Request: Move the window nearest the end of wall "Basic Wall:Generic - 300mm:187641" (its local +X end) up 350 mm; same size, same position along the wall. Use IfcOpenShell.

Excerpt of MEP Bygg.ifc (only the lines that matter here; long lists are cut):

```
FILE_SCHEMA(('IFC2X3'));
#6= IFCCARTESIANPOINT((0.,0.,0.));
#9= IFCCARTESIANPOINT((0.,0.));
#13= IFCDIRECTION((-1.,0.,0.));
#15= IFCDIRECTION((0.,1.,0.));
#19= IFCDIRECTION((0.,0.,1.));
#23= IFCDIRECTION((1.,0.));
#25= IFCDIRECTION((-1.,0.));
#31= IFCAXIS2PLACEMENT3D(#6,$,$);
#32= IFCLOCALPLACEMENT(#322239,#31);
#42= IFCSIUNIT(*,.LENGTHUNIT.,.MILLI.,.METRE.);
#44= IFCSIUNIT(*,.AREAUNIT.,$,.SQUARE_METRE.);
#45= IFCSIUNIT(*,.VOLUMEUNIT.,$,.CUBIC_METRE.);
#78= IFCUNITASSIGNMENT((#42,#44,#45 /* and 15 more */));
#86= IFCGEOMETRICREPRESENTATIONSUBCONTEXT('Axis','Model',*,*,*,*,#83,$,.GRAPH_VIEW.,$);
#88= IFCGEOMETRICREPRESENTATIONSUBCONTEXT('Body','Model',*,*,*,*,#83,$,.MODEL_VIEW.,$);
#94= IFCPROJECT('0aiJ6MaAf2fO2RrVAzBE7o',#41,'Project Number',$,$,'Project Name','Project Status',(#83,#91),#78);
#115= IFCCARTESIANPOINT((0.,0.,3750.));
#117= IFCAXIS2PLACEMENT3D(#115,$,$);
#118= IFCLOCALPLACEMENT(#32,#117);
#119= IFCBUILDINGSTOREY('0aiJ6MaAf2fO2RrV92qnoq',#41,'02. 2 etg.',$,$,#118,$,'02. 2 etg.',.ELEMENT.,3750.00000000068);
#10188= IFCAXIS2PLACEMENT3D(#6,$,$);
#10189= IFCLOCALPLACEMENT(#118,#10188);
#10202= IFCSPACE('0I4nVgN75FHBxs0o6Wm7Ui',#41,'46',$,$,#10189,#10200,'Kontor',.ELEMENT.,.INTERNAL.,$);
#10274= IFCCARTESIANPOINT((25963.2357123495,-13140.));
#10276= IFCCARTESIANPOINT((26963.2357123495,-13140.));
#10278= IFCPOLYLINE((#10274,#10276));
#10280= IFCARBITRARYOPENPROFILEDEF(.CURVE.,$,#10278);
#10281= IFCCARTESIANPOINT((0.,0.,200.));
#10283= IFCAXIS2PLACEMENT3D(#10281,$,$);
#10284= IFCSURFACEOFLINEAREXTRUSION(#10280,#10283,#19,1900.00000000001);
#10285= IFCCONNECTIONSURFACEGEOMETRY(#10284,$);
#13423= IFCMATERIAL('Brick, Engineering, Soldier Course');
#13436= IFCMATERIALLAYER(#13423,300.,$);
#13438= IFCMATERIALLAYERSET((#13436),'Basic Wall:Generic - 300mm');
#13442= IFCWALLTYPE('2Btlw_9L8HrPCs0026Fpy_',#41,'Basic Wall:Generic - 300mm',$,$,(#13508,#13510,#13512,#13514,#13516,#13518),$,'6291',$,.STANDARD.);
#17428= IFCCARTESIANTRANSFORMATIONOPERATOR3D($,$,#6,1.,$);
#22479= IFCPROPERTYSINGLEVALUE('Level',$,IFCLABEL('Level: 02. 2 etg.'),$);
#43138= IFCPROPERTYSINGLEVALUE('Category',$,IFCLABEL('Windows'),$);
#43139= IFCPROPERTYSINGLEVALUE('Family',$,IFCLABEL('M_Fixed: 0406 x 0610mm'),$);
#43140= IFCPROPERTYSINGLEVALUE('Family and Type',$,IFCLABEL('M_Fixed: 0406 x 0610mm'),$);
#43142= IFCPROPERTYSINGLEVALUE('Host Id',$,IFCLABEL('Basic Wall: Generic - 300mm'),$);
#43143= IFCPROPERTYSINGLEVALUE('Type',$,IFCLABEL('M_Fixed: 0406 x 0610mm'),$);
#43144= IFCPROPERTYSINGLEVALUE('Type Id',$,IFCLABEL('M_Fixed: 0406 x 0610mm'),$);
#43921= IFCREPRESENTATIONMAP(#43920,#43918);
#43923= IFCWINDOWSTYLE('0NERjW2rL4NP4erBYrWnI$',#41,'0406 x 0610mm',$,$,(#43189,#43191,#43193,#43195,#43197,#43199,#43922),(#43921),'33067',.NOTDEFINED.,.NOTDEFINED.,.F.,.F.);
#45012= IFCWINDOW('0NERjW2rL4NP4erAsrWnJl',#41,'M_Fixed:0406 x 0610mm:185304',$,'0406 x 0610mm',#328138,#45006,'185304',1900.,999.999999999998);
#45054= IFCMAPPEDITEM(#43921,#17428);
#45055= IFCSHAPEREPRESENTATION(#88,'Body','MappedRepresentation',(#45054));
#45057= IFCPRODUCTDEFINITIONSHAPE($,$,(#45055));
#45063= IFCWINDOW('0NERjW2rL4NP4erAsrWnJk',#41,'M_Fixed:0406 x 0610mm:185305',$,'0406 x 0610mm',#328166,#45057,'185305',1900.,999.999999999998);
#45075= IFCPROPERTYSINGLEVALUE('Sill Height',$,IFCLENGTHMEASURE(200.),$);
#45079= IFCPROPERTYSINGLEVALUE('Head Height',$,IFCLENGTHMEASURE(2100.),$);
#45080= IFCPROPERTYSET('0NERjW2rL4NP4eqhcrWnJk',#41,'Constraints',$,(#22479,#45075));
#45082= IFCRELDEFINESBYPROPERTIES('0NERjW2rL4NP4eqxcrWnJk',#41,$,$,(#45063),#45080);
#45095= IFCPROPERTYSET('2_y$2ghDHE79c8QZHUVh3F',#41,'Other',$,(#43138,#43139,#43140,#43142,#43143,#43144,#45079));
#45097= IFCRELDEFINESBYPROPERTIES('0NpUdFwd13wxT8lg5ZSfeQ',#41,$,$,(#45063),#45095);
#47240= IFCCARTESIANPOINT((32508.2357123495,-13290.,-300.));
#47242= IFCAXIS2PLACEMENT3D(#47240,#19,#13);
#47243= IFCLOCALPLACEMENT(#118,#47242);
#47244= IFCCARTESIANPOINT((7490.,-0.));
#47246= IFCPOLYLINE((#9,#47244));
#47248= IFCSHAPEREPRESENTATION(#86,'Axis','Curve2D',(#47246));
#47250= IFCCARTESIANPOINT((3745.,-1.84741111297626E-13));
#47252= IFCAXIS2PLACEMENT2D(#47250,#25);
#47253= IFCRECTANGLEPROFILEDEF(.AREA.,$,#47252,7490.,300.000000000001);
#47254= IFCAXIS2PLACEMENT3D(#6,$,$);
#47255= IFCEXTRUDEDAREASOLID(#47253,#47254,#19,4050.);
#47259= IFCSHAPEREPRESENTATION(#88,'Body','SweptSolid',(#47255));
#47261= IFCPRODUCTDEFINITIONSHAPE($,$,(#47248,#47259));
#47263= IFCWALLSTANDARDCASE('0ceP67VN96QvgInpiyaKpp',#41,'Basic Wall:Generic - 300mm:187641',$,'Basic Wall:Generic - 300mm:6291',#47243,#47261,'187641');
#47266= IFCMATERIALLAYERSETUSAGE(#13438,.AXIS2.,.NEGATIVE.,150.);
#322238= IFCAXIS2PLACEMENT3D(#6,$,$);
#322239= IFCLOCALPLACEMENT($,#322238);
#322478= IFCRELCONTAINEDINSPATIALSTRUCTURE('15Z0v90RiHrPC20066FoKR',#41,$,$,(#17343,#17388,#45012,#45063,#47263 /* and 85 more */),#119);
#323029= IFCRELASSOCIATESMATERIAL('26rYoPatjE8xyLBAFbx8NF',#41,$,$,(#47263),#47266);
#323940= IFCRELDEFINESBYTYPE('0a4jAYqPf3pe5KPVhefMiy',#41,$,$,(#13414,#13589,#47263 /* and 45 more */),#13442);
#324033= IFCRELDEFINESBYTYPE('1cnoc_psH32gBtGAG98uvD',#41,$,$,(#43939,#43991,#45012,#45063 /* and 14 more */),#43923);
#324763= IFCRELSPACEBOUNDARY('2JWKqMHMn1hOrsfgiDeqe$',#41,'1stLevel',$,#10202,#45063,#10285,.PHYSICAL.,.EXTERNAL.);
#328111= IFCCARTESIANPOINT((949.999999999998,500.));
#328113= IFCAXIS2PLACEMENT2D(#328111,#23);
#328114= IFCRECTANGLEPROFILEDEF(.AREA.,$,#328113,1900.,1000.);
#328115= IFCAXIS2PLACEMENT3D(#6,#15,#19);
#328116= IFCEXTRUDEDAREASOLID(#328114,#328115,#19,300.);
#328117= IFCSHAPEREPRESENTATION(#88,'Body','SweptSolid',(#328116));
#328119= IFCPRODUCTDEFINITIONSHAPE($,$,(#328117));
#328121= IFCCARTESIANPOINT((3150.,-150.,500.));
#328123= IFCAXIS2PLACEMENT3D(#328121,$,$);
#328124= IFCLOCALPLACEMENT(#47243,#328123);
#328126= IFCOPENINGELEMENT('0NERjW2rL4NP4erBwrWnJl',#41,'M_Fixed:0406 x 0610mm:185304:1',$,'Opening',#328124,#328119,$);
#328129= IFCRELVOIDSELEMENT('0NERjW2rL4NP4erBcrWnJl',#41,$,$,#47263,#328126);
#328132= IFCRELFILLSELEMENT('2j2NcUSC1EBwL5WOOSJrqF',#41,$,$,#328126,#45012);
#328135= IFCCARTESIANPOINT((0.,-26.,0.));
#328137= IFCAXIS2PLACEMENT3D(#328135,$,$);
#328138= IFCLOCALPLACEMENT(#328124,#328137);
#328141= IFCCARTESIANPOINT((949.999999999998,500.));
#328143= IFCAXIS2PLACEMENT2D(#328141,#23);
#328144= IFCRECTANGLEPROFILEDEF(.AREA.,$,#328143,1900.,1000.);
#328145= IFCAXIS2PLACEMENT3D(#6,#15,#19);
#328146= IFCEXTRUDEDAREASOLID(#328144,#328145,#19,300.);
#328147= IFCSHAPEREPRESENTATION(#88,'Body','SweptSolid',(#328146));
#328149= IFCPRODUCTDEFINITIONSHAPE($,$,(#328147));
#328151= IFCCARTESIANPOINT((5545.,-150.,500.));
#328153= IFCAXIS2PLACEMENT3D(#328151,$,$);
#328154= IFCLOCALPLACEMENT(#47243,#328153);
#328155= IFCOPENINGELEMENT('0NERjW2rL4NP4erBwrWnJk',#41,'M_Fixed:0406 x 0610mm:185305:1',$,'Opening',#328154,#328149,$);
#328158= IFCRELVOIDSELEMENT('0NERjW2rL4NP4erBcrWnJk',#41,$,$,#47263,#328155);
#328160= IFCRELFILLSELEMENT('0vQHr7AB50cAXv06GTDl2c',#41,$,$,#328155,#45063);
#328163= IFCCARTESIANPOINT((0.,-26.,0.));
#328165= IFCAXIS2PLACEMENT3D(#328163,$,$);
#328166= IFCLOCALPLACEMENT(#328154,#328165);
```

```python
import numpy as np
import ifcopenshell
import ifcopenshell.api.geometry
import ifcopenshell.api.pset
import ifcopenshell.util.element
import ifcopenshell.util.placement
import ifcopenshell.util.unit

model = ifcopenshell.open("MEP Bygg.ifc")
unit_scale = ifcopenshell.util.unit.calculate_unit_scale(model)

window = model.by_guid("0NERjW2rL4NP4erAsrWnJk")
opening = window.FillsVoids[0].RelatingOpeningElement
dz = 0.35 / unit_scale

shift = np.array([0.0, 0.0, dz])
# The window is placed relative to its opening, so it follows when the opening moves.
matrix = ifcopenshell.util.placement.get_local_placement(opening.ObjectPlacement)
matrix[:3, 3] += shift
ifcopenshell.api.geometry.edit_object_placement(
    model, product=opening, matrix=matrix, is_si=False, should_transform_children=True
)

# Space boundary surfaces are stored in each space's coordinates; move them too.
for rel in window.ProvidesBoundaries:
    if not rel.ConnectionGeometry:
        continue
    surface = rel.ConnectionGeometry.SurfaceOnRelatingElement
    space_matrix = ifcopenshell.util.placement.get_local_placement(rel.RelatingSpace.ObjectPlacement)
    point = np.array(surface.Position.Location.Coordinates) + space_matrix[:3, :3].T @ shift
    surface.Position = model.createIfcAxis2Placement3D(
        model.createIfcCartesianPoint(point.tolist()), surface.Position.Axis, surface.Position.RefDirection
    )

# Keep the stored heights in step.
pset = model.by_id(ifcopenshell.util.element.get_pset(window, "Constraints", should_inherit=False)["id"])
ifcopenshell.api.pset.edit_pset(model, pset=pset, properties={
    "Sill Height": model.create_entity("IfcLengthMeasure", ifcopenshell.util.element.get_pset(window, "Constraints", "Sill Height") + dz),
})
pset = model.by_id(ifcopenshell.util.element.get_pset(window, "Other", should_inherit=False)["id"])
ifcopenshell.api.pset.edit_pset(model, pset=pset, properties={
    "Head Height": model.create_entity("IfcLengthMeasure", ifcopenshell.util.element.get_pset(window, "Other", "Head Height") + dz),
})

print(f"moved by {dz * unit_scale:+.3f} m")

model.write("MEP Bygg_rev.ifc")
```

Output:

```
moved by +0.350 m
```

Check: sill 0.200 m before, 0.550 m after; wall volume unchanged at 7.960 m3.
